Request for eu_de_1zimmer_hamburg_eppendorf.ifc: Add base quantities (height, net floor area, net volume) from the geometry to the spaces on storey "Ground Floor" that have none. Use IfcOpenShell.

First a look at what the model holds.

```python
import ifcopenshell
import ifcopenshell.util.element
import ifcopenshell.util.unit

model = ifcopenshell.open("eu_de_1zimmer_hamburg_eppendorf.ifc")
print(model.schema)
for unit_type in ("LENGTHUNIT", "AREAUNIT", "VOLUMEUNIT"):
    print(unit_type, ifcopenshell.util.unit.calculate_unit_scale(model, unit_type))
storey = next(s for s in model.by_type("IfcBuildingStorey") if s.Name == "Ground Floor")
spaces = [e for e in ifcopenshell.util.element.get_decomposition(storey) if e.is_a("IfcSpace")]
for e in sorted(spaces, key=lambda e: e.id()):
    print(e.id(), e.is_a(), e.Name, list(ifcopenshell.util.element.get_psets(e, qtos_only=True)), sep=" | ")
```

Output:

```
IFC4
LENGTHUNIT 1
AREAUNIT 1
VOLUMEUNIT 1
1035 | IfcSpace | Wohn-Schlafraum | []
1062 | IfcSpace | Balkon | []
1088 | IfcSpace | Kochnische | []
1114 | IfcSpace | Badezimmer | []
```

```python
import ifcopenshell
import ifcopenshell.api.pset
import ifcopenshell.geom
import ifcopenshell.util.element
import ifcopenshell.util.shape
import ifcopenshell.util.unit

model = ifcopenshell.open("eu_de_1zimmer_hamburg_eppendorf.ifc")
unit_scale = ifcopenshell.util.unit.calculate_unit_scale(model)
area_scale = ifcopenshell.util.unit.calculate_unit_scale(model, "AREAUNIT")
volume_scale = ifcopenshell.util.unit.calculate_unit_scale(model, "VOLUMEUNIT")
settings = ifcopenshell.geom.settings()

storey = next(s for s in model.by_type("IfcBuildingStorey") if s.Name == "Ground Floor")
spaces = [e for e in ifcopenshell.util.element.get_decomposition(storey) if e.is_a("IfcSpace")]

for e in sorted(spaces, key=lambda e: e.id()):
    if ifcopenshell.util.element.get_psets(e, qtos_only=True, should_inherit=False):
        continue
    # Geometry comes back in metres, in the element's own axes.
    shape = ifcopenshell.geom.create_shape(settings, e)
    values = {
        "Height": ifcopenshell.util.shape.get_z(shape.geometry) / unit_scale,
        "NetFloorArea": ifcopenshell.util.shape.get_footprint_area(shape.geometry) / area_scale,
        "NetVolume": ifcopenshell.util.shape.get_volume(shape.geometry) / volume_scale,
    }
    qto = ifcopenshell.api.pset.add_qto(model, product=e, name="Qto_SpaceBaseQuantities")
    ifcopenshell.api.pset.edit_qto(model, qto=qto, properties=values)
    print(e.id(), {k: round(v, 3) for k, v in values.items()})

model.write("eu_de_1zimmer_hamburg_eppendorf_v2.ifc")
```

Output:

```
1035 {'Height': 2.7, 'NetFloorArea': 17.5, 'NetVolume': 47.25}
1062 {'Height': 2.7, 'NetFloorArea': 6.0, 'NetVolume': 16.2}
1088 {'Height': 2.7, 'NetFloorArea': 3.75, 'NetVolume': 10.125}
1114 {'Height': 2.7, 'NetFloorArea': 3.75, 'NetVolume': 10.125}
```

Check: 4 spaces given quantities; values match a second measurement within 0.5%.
